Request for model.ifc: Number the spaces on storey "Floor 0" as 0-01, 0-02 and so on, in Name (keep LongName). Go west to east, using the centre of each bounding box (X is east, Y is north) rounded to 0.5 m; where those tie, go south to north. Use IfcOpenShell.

First a look at what the model holds.

```python
import ifcopenshell
import ifcopenshell.util.element
import ifcopenshell.util.placement

model = ifcopenshell.open("model.ifc")
print(model.schema)
storey = next(s for s in model.by_type("IfcBuildingStorey") if s.Name == "Floor 0")
spaces = [e for e in ifcopenshell.util.element.get_decomposition(storey) if e.is_a("IfcSpace")]
for e in sorted(spaces, key=lambda e: e.id()):
    origin = ifcopenshell.util.placement.get_local_placement(e.ObjectPlacement)[:3, 3]
    print(e.id(), e.Name, e.LongName, origin.round(2) + 0.0, sep=" | ")
```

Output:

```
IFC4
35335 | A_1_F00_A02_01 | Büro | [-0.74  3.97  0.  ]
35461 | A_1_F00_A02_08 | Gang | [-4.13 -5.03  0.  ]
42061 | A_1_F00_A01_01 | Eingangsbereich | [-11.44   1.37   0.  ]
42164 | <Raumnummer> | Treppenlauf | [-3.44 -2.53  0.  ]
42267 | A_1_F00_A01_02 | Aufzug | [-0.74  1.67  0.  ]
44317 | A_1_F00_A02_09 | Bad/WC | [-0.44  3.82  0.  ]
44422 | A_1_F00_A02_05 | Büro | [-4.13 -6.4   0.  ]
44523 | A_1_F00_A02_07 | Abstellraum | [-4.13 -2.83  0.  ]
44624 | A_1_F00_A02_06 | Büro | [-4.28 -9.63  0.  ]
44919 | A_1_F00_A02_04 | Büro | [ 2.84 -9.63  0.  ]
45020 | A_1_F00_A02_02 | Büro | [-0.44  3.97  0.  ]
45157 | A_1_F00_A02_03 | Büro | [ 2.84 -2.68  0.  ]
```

```python
import ifcopenshell
import ifcopenshell.geom
import ifcopenshell.util.element
import ifcopenshell.util.shape

model = ifcopenshell.open("model.ifc")
settings = ifcopenshell.geom.settings()
settings.set("use-world-coords", True)


def centre(element):
    shape = ifcopenshell.geom.create_shape(settings, element)
    return ifcopenshell.util.shape.get_bbox_centroid(shape.geometry)


storey = next(s for s in model.by_type("IfcBuildingStorey") if s.Name == "Floor 0")
spaces = [e for e in ifcopenshell.util.element.get_decomposition(storey) if e.is_a("IfcSpace")]

# Insertion points can sit at a corner or the storey origin, so sort by the geometry (in metres).
centres = {e: centre(e) for e in spaces}
spaces.sort(key=lambda e: (round(centres[e][0] / 0.5), centres[e][1]))

for i, e in enumerate(spaces, start=1):
    number = f"0-{i:02d}"
    e.Name = number
    print(e.id(), number)

model.write("model-out.ifc")
```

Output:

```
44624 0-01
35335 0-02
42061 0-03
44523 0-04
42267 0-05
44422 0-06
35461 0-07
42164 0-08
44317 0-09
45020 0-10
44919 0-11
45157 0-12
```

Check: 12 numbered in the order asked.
